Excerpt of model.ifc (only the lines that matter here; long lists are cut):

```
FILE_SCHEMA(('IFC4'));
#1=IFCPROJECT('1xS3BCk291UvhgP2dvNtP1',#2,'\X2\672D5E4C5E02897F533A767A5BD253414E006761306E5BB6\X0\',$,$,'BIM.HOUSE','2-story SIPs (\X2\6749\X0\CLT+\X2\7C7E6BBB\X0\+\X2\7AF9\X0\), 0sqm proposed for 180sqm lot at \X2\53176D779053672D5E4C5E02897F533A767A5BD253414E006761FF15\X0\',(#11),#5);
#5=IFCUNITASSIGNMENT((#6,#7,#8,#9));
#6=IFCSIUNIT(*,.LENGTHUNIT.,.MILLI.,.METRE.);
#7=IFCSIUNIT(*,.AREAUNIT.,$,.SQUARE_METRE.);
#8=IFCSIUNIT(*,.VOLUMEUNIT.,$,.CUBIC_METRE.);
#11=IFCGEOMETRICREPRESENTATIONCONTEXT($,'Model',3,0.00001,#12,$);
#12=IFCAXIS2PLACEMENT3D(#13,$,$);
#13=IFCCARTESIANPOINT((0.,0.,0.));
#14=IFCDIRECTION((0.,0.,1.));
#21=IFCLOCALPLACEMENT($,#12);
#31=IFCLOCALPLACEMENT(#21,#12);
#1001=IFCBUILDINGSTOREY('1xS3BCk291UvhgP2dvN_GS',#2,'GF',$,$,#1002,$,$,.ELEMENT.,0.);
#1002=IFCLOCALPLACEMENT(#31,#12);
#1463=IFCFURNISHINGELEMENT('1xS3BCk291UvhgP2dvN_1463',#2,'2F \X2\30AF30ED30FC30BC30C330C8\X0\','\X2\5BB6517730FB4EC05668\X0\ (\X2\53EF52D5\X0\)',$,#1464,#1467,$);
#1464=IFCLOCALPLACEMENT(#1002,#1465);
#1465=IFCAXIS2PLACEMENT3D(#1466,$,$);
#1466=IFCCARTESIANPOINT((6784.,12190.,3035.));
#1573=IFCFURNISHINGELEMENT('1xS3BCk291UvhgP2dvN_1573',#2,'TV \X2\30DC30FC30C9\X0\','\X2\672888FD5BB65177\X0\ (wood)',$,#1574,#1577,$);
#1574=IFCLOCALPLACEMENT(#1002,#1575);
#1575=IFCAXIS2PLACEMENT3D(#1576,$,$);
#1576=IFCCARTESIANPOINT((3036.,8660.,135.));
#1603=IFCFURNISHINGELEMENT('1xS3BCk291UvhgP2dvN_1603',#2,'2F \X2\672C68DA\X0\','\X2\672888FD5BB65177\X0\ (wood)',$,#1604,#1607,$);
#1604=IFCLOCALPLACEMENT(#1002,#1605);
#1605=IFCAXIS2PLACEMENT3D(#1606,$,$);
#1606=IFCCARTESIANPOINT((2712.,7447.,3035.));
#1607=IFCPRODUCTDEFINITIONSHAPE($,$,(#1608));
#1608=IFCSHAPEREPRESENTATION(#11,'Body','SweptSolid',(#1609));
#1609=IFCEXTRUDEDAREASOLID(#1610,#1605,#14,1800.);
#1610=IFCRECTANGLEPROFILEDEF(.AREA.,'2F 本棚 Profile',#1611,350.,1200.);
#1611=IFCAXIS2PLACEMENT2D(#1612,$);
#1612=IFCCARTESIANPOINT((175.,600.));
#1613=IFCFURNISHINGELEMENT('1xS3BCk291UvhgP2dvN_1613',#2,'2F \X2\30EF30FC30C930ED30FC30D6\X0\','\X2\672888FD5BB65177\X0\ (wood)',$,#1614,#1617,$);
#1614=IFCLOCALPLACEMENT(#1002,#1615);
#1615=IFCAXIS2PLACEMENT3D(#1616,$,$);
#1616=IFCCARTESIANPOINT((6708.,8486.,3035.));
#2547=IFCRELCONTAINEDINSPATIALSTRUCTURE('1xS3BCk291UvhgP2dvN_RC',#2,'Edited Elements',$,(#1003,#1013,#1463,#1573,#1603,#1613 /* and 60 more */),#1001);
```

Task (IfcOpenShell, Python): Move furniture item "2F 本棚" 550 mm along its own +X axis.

```python
import ifcopenshell
import ifcopenshell.api.geometry
import ifcopenshell.util.placement
import ifcopenshell.util.unit

model = ifcopenshell.open("model.ifc")
unit_scale = ifcopenshell.util.unit.calculate_unit_scale(model)

item = model.by_guid("1xS3BCk291UvhgP2dvN_1603")
matrix = ifcopenshell.util.placement.get_local_placement(item.ObjectPlacement)
matrix[:3, 3] += matrix[:3, 0] * 0.55 / unit_scale
ifcopenshell.api.geometry.edit_object_placement(model, product=item, matrix=matrix, is_si=False)

print(ifcopenshell.util.placement.get_local_placement(item.ObjectPlacement).round(3) + 0.0)

model.write("model_rev.ifc")
```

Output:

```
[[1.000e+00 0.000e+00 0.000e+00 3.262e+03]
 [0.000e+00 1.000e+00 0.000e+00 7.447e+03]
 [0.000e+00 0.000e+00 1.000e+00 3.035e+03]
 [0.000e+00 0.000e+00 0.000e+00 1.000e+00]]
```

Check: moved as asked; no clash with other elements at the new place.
